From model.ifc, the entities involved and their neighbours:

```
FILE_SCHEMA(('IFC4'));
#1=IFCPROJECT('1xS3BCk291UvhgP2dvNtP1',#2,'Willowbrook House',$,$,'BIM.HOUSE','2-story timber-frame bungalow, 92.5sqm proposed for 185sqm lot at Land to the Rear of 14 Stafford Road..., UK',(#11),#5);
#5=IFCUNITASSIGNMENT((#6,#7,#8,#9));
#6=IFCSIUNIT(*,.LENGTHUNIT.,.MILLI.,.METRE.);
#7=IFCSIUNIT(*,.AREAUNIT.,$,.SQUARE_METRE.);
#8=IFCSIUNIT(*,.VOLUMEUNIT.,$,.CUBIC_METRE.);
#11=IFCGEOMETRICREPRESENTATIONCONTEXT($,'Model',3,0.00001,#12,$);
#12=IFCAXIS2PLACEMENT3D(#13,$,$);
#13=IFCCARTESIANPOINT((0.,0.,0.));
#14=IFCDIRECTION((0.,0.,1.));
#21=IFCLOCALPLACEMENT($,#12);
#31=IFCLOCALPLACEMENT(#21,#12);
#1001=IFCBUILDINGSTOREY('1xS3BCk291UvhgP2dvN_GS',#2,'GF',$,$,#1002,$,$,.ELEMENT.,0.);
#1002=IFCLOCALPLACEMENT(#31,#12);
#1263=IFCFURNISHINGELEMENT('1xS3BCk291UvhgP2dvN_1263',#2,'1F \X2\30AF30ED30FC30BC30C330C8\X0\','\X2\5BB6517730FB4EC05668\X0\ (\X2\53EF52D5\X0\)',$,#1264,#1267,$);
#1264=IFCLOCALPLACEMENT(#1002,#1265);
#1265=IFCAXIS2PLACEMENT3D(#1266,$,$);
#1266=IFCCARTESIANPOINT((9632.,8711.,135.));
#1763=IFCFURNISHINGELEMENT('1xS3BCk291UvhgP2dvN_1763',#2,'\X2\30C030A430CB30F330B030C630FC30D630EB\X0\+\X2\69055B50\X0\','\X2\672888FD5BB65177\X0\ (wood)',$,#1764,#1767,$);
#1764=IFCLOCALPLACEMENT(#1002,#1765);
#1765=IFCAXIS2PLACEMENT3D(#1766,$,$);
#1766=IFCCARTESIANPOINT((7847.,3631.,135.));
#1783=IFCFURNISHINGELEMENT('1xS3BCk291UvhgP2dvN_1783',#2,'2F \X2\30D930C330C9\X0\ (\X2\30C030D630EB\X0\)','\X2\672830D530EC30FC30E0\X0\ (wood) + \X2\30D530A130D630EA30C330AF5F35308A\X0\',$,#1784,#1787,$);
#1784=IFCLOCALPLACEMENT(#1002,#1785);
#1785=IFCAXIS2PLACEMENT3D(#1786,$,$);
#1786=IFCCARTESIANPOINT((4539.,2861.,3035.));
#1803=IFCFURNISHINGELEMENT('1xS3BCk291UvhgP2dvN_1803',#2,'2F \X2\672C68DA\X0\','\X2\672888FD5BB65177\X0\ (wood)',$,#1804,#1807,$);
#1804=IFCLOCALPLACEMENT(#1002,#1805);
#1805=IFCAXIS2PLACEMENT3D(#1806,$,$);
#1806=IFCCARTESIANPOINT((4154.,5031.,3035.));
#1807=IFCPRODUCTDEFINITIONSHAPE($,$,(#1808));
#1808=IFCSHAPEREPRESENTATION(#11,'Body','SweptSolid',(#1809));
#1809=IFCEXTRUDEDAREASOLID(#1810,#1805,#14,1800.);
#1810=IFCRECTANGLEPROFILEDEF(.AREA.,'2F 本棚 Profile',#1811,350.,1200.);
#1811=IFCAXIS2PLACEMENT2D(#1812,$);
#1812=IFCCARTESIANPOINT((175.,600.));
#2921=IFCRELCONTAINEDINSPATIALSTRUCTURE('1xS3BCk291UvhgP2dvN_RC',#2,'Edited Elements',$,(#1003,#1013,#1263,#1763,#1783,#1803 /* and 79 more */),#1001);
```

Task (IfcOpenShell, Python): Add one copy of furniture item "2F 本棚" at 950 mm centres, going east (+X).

```python
import numpy as np
import ifcopenshell
import ifcopenshell.api.geometry
import ifcopenshell.api.root
import ifcopenshell.util.element
import ifcopenshell.util.placement
import ifcopenshell.util.unit

model = ifcopenshell.open("model.ifc")
unit_scale = ifcopenshell.util.unit.calculate_unit_scale(model)


def reuse_history(source, copy):
    """copy_class also copies each property set's owner history, people and application; keep the originals."""
    for rel in copy.IsDefinedBy:
        if rel.is_a("IfcRelDefinesByProperties") and (history := rel.RelatingPropertyDefinition.OwnerHistory):
            rel.RelatingPropertyDefinition.OwnerHistory = source.OwnerHistory
            ifcopenshell.util.element.remove_deep2(model, history)


source = model.by_guid("1xS3BCk291UvhgP2dvN_1803")
base = ifcopenshell.util.placement.get_local_placement(source.ObjectPlacement)
step = np.array([1.0, 0.0, 0.0]) * 0.95 / unit_scale

for i in range(1, 2):
    copy = ifcopenshell.api.root.copy_class(model, product=source)
    copy.Representation = ifcopenshell.util.element.copy_deep(
        model, source.Representation, exclude=["IfcGeometricRepresentationContext", "IfcRepresentationMap"]
    )
    reuse_history(source, copy)
    matrix = base.copy()
    matrix[:3, 3] += i * step
    print("added at", matrix[:3, 3].round(3) + 0.0)
    ifcopenshell.api.geometry.edit_object_placement(model, product=copy, matrix=matrix, is_si=False)

model.write("model_v2.ifc")
```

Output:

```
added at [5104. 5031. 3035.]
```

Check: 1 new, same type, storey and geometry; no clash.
